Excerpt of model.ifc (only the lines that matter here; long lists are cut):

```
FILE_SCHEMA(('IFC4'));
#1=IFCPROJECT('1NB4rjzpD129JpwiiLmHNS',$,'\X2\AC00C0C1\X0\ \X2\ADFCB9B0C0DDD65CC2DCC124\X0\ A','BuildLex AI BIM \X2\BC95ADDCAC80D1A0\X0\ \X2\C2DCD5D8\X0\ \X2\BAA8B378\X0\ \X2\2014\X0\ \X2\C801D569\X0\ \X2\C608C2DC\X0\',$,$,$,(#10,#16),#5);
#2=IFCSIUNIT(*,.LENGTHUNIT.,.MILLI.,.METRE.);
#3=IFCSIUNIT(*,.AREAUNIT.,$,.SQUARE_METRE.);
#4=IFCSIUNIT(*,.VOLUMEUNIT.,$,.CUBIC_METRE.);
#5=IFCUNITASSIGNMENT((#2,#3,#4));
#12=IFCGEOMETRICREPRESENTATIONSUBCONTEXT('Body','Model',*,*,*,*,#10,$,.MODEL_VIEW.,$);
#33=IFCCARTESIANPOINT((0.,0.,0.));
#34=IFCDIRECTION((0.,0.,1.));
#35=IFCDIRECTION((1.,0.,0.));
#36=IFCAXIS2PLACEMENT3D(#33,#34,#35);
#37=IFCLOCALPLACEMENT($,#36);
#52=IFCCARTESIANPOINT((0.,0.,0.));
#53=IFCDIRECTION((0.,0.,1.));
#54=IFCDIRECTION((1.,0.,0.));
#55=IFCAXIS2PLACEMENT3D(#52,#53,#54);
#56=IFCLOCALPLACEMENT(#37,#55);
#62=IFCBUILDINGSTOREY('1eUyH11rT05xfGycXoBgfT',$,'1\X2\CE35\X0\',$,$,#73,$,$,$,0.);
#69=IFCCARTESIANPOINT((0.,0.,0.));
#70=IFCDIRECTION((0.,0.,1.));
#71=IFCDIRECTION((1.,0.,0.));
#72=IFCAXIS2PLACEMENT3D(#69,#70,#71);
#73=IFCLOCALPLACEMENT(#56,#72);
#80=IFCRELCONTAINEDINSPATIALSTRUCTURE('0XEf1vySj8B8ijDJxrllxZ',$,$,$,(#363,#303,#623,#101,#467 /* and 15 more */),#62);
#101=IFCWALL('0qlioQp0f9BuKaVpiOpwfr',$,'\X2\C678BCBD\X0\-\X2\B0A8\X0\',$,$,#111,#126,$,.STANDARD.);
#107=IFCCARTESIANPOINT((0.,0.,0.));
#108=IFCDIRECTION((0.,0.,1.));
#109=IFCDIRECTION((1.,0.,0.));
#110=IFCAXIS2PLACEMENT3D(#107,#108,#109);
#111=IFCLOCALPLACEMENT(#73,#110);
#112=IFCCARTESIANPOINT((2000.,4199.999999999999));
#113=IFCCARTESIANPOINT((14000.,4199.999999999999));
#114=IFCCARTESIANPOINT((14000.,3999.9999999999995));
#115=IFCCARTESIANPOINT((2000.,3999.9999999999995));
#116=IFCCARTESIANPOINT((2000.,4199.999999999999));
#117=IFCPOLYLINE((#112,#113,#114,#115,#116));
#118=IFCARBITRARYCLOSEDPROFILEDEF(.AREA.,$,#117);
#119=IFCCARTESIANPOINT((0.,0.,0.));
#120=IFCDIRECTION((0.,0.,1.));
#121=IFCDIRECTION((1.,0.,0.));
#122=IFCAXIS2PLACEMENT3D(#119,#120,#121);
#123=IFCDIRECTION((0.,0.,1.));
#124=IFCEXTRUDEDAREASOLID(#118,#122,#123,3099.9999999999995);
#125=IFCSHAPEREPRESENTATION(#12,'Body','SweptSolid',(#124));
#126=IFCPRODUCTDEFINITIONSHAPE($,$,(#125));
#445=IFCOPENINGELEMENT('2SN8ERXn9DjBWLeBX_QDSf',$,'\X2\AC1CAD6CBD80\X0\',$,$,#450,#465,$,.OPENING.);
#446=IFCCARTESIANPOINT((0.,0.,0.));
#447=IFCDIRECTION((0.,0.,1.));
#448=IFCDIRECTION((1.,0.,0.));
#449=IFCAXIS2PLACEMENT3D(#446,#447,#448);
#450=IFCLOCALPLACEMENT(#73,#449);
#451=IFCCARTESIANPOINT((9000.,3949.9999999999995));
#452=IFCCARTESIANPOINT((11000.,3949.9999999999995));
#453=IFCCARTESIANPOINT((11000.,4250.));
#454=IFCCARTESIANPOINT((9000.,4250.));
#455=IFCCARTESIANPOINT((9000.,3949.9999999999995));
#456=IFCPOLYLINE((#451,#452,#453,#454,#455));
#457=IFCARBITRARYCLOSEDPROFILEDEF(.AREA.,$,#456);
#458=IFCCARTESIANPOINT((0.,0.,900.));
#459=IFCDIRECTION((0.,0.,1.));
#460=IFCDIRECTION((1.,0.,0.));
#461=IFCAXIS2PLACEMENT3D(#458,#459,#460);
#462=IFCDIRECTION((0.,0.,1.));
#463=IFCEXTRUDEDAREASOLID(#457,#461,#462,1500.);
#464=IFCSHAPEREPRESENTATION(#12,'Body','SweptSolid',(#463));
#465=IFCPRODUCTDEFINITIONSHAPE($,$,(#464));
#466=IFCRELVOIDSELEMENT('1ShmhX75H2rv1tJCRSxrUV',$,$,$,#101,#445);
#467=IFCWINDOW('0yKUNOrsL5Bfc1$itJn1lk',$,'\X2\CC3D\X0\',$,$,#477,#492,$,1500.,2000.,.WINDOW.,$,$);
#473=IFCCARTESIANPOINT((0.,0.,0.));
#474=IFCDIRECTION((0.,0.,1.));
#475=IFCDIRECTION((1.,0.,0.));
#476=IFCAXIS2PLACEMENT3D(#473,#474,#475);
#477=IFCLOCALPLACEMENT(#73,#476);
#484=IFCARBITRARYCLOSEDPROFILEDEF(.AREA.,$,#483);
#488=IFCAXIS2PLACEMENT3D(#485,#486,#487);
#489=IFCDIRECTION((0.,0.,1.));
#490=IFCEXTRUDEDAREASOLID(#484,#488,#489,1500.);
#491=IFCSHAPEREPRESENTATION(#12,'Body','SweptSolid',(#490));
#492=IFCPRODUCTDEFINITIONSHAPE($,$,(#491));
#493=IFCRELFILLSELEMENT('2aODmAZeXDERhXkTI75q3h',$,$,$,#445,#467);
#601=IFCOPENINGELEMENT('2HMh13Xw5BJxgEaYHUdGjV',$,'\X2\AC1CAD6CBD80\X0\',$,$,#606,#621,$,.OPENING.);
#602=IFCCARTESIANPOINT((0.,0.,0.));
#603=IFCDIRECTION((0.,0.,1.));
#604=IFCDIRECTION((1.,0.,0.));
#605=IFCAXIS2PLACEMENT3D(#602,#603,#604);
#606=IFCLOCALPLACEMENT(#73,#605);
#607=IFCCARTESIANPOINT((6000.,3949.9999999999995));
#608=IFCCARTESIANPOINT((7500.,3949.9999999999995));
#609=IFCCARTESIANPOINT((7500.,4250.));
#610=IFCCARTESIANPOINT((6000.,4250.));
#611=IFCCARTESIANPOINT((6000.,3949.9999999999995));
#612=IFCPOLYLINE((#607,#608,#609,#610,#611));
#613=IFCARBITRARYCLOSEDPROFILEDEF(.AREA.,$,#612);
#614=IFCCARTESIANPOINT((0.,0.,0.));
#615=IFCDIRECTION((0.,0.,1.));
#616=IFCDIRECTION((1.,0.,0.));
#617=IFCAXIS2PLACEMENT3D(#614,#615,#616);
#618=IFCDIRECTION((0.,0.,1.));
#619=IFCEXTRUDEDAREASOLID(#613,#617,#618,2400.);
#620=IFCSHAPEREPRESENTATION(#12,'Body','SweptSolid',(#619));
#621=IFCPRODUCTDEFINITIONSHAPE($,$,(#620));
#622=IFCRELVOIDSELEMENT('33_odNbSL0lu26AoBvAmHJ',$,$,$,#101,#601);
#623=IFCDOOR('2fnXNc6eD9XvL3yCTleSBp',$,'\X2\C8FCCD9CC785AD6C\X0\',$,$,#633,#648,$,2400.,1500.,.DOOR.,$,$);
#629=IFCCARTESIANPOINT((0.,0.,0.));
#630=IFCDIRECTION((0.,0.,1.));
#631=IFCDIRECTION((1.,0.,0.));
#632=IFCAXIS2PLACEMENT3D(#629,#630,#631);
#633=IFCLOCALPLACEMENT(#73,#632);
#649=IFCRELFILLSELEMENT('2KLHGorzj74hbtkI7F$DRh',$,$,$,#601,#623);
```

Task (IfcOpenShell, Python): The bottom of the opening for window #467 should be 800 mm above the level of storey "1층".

```python
import numpy as np
import ifcopenshell
import ifcopenshell.api.geometry
import ifcopenshell.geom
import ifcopenshell.util.element
import ifcopenshell.util.placement
import ifcopenshell.util.shape
import ifcopenshell.util.unit

model = ifcopenshell.open("model.ifc")
unit_scale = ifcopenshell.util.unit.calculate_unit_scale(model)

window = model.by_guid("0yKUNOrsL5Bfc1$itJn1lk")
opening = window.FillsVoids[0].RelatingOpeningElement
storey = ifcopenshell.util.element.get_container(window, ifc_class="IfcBuildingStorey")
level = ifcopenshell.util.placement.get_local_placement(storey.ObjectPlacement)[2, 3]

# The opening's origin need not be at the sill, so measure its lowest point.
shape = ifcopenshell.geom.create_shape(ifcopenshell.geom.settings(), opening)
bottom = ifcopenshell.util.shape.get_shape_bottom_elevation(shape, shape.geometry) / unit_scale
dz = level + 800.0 - bottom

shift = np.array([0.0, 0.0, dz])
# The window is not placed relative to its opening, so move both.
for product in (opening, window):
    matrix = ifcopenshell.util.placement.get_local_placement(product.ObjectPlacement)
    matrix[:3, 3] += shift
    ifcopenshell.api.geometry.edit_object_placement(model, product=product, matrix=matrix, is_si=False)

print(f"moved by {dz * unit_scale:+.3f} m")

model.write("model_updated.ifc")
```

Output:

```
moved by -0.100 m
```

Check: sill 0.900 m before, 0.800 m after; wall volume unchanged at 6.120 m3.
